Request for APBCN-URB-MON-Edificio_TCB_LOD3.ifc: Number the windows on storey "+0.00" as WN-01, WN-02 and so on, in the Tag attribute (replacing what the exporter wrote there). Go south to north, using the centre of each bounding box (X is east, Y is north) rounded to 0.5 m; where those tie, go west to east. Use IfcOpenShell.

First a look at what the model holds.

```python
import ifcopenshell
import ifcopenshell.util.element
import ifcopenshell.util.placement

model = ifcopenshell.open("APBCN-URB-MON-Edificio_TCB_LOD3.ifc")
print(model.schema)
storey = next(s for s in model.by_type("IfcBuildingStorey") if s.Name == "+0.00")
windows = [e for e in ifcopenshell.util.element.get_decomposition(storey) if e.is_a("IfcWindow")]
for e in sorted(windows, key=lambda e: e.id()):
    origin = ifcopenshell.util.placement.get_local_placement(e.ObjectPlacement)[:3, 3]
    print(e.id(), e.Tag, e.Name, origin.round(2) + 0.0, sep=" | ")
```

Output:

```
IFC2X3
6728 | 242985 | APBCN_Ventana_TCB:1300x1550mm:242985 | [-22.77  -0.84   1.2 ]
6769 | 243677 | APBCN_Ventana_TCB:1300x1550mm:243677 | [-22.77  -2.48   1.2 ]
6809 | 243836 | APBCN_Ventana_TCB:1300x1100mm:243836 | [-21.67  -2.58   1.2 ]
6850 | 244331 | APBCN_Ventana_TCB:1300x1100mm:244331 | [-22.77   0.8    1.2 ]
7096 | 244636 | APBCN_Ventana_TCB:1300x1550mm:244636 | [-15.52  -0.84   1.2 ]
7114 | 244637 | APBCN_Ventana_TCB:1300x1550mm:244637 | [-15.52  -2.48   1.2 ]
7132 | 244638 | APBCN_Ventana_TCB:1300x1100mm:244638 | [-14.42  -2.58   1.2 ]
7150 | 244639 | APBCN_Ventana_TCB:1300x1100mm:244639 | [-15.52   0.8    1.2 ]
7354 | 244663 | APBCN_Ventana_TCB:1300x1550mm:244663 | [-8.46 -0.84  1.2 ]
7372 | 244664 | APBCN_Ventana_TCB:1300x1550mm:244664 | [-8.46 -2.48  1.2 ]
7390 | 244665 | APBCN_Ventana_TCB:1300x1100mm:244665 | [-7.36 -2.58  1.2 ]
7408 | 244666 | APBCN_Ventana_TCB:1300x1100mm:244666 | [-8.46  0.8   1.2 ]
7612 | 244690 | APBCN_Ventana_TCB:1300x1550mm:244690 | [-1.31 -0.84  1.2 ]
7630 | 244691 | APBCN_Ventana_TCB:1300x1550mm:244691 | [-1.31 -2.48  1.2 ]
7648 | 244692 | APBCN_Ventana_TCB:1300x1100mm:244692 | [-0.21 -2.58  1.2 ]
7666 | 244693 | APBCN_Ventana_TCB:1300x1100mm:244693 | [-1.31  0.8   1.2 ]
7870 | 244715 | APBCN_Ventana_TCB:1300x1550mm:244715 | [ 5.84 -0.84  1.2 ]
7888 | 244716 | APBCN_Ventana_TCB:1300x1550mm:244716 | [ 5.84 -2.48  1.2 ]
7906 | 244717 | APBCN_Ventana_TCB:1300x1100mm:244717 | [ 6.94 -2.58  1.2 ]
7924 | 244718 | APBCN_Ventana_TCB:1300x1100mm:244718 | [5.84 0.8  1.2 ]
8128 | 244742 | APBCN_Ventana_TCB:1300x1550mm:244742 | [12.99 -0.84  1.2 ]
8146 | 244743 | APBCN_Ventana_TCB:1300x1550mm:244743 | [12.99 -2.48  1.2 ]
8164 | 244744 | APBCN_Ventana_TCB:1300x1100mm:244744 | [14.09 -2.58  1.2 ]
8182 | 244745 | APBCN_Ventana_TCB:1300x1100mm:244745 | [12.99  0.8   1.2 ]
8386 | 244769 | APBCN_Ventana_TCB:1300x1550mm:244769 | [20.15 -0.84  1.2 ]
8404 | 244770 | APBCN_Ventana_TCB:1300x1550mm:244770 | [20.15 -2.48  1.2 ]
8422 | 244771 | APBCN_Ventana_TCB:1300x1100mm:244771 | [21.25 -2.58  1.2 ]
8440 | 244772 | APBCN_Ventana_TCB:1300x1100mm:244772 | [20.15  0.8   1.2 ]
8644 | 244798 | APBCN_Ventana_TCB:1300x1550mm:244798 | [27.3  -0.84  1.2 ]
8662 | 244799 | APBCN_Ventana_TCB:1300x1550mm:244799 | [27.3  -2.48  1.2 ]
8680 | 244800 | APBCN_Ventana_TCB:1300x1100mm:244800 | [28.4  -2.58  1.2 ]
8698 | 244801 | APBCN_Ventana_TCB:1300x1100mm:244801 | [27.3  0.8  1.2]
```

```python
import ifcopenshell
import ifcopenshell.geom
import ifcopenshell.util.element
import ifcopenshell.util.shape

model = ifcopenshell.open("APBCN-URB-MON-Edificio_TCB_LOD3.ifc")
settings = ifcopenshell.geom.settings()
settings.set("use-world-coords", True)


def centre(element):
    shape = ifcopenshell.geom.create_shape(settings, element)
    return ifcopenshell.util.shape.get_bbox_centroid(shape.geometry)


storey = next(s for s in model.by_type("IfcBuildingStorey") if s.Name == "+0.00")
windows = [e for e in ifcopenshell.util.element.get_decomposition(storey) if e.is_a("IfcWindow")]

# Insertion points can sit at a corner or the storey origin, so sort by the geometry (in metres).
centres = {e: centre(e) for e in windows}
windows.sort(key=lambda e: (round(centres[e][1] / 0.5), centres[e][0]))

for i, e in enumerate(windows, start=1):
    number = f"WN-{i:02d}"
    e.Tag = number
    print(e.id(), number)

model.write("APBCN-URB-MON-Edificio_TCB_LOD3_edited.ifc")
```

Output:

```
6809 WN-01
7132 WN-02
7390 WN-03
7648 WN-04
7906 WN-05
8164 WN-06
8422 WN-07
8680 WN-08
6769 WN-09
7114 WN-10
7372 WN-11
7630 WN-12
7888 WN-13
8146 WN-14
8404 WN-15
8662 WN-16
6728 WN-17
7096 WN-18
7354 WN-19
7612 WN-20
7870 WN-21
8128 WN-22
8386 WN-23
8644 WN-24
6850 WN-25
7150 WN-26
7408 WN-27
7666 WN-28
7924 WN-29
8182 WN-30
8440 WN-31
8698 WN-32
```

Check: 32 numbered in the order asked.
